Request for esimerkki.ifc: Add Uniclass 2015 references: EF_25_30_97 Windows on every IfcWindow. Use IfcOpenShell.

First a look at what the model holds.

```python
import ifcopenshell

model = ifcopenshell.open("esimerkki.ifc")
print(model.schema)
print("classifications:", [c.Name for c in model.by_type("IfcClassification")])
for ifc_class in ("IfcDoor", "IfcRoof", "IfcStair", "IfcWall", "IfcWindow"):
    print(ifc_class, len(model.by_type(ifc_class)))
```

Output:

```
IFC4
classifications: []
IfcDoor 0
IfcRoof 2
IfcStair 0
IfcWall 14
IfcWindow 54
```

```python
import ifcopenshell
import ifcopenshell.api.classification

model = ifcopenshell.open("esimerkki.ifc")

system = ifcopenshell.api.classification.add_classification(model, classification="Uniclass 2015")

codes = {
    "IfcWindow": ("EF_25_30_97", "Windows"),
}
for ifc_class, (code, name) in codes.items():
    products = model.by_type(ifc_class)
    ifcopenshell.api.classification.add_reference(
        model, products=products, classification=system, identification=code, name=name
    )
    print(code, len(products))

model.write("esimerkki_updated.ifc")
```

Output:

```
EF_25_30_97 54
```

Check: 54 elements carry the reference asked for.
